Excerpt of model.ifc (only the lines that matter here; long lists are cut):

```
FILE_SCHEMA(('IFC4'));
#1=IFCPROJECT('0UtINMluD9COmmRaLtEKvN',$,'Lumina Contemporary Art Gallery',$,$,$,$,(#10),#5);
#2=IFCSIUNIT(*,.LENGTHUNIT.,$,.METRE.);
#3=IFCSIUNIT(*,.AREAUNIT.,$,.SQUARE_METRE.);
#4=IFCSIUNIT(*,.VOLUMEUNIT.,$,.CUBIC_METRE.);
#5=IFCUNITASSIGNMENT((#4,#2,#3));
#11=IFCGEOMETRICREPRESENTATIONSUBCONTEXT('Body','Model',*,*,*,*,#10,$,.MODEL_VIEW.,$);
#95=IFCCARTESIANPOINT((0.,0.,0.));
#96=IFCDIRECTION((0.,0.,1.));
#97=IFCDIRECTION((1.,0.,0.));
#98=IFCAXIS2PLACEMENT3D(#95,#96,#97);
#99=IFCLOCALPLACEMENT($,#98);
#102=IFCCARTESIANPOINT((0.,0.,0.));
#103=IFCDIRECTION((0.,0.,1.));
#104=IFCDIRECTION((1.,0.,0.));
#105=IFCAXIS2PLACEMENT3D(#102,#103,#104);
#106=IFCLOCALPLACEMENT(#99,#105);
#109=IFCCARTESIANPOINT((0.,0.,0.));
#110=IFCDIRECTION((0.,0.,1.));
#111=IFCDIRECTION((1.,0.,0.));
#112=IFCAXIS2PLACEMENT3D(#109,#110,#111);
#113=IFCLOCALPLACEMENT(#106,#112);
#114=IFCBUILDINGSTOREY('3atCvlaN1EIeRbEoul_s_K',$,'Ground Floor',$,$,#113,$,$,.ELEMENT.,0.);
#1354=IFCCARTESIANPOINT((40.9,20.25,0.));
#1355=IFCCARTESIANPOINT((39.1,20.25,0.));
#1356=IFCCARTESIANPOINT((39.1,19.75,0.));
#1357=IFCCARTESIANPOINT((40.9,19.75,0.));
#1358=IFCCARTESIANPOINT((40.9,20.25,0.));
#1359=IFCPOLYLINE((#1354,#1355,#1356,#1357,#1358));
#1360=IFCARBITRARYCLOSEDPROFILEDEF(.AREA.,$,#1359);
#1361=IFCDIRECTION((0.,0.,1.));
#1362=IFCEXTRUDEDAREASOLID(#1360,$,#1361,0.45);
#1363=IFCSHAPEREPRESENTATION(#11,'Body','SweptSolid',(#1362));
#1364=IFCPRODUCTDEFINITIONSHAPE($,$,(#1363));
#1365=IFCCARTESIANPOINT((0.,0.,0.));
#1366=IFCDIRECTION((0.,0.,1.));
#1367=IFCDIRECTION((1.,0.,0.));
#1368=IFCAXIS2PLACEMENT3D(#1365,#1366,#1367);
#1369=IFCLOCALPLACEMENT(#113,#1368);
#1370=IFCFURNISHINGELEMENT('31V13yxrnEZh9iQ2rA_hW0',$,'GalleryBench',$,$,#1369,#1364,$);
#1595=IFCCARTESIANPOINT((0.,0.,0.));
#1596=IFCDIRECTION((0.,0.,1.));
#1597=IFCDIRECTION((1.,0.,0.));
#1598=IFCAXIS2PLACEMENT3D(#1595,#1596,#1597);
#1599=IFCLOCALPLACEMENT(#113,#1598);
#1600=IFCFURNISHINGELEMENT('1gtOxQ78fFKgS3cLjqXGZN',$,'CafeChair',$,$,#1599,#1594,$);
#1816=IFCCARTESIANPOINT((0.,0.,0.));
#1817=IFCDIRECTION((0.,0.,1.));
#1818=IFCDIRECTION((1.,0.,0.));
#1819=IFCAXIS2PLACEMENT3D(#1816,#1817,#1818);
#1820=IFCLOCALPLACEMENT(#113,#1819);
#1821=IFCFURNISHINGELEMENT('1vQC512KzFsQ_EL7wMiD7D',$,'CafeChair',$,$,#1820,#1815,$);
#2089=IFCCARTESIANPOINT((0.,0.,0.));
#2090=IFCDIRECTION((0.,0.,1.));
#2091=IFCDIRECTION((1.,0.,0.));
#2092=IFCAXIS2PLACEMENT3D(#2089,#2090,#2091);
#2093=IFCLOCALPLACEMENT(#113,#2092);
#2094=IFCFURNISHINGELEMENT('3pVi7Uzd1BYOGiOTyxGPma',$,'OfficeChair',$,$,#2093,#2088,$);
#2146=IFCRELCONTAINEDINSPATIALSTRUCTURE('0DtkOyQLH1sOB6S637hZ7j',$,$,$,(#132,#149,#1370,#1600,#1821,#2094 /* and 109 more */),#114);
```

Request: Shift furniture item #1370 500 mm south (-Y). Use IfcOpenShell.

```python
import ifcopenshell
import ifcopenshell.api.geometry
import ifcopenshell.util.placement

model = ifcopenshell.open("model.ifc")

item = model.by_id(1370)
matrix = ifcopenshell.util.placement.get_local_placement(item.ObjectPlacement)
matrix[1, 3] -= 0.5
ifcopenshell.api.geometry.edit_object_placement(model, product=item, matrix=matrix, is_si=False)

print(ifcopenshell.util.placement.get_local_placement(item.ObjectPlacement).round(3) + 0.0)

model.write("model-out.ifc")
```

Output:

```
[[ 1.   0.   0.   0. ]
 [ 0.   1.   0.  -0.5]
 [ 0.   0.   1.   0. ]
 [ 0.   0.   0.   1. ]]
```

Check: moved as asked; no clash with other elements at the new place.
